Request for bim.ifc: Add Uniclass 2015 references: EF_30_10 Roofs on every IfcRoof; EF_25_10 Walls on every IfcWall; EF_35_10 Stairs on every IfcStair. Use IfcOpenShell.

First a look at what the model holds.

```python
import ifcopenshell

model = ifcopenshell.open("bim.ifc")
print(model.schema)
print("classifications:", [c.Name for c in model.by_type("IfcClassification")])
for ifc_class in ("IfcDoor", "IfcRoof", "IfcStair", "IfcWall", "IfcWindow"):
    print(ifc_class, len(model.by_type(ifc_class)))
```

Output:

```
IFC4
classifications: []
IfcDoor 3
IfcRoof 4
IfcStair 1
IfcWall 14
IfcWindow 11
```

```python
import ifcopenshell
import ifcopenshell.api.classification

model = ifcopenshell.open("bim.ifc")

system = ifcopenshell.api.classification.add_classification(model, classification="Uniclass 2015")

codes = {
    "IfcRoof": ("EF_30_10", "Roofs"),
    "IfcWall": ("EF_25_10", "Walls"),
    "IfcStair": ("EF_35_10", "Stairs"),
}
for ifc_class, (code, name) in codes.items():
    products = model.by_type(ifc_class)
    ifcopenshell.api.classification.add_reference(
        model, products=products, classification=system, identification=code, name=name
    )
    print(code, len(products))

model.write("bim_edited.ifc")
```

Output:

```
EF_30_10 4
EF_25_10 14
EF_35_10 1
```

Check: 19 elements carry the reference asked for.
